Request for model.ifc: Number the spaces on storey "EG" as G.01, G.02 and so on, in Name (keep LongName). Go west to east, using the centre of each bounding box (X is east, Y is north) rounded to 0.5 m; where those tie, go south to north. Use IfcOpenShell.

First a look at what the model holds.

```python
import ifcopenshell
import ifcopenshell.util.element
import ifcopenshell.util.placement

model = ifcopenshell.open("model.ifc")
print(model.schema)
storey = next(s for s in model.by_type("IfcBuildingStorey") if s.Name == "EG")
spaces = [e for e in ifcopenshell.util.element.get_decomposition(storey) if e.is_a("IfcSpace")]
for e in sorted(spaces, key=lambda e: e.id()):
    origin = ifcopenshell.util.placement.get_local_placement(e.ObjectPlacement)[:3, 3]
    print(e.id(), e.Name, e.LongName, origin.round(2) + 0.0, sep=" | ")
```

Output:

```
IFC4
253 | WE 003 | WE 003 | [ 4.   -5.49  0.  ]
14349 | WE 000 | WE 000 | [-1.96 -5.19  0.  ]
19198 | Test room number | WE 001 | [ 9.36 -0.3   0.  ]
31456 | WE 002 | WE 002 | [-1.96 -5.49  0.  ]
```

```python
import ifcopenshell
import ifcopenshell.geom
import ifcopenshell.util.element
import ifcopenshell.util.shape

model = ifcopenshell.open("model.ifc")
settings = ifcopenshell.geom.settings()
settings.set("use-world-coords", True)


def centre(element):
    shape = ifcopenshell.geom.create_shape(settings, element)
    return ifcopenshell.util.shape.get_bbox_centroid(shape.geometry)


storey = next(s for s in model.by_type("IfcBuildingStorey") if s.Name == "EG")
spaces = [e for e in ifcopenshell.util.element.get_decomposition(storey) if e.is_a("IfcSpace")]

# Insertion points can sit at a corner or the storey origin, so sort by the geometry (in metres).
centres = {e: centre(e) for e in spaces}
spaces.sort(key=lambda e: (round(centres[e][0] / 0.5), centres[e][1]))

for i, e in enumerate(spaces, start=1):
    number = f"G.{i:02d}"
    e.Name = number
    print(e.id(), number)

model.write("model-out.ifc")
```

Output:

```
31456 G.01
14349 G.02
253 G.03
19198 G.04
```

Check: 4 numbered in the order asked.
